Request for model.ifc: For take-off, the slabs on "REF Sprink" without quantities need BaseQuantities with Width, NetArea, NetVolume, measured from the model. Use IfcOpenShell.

First a look at what the model holds.

```python
import ifcopenshell
import ifcopenshell.util.element
import ifcopenshell.util.unit

model = ifcopenshell.open("model.ifc")
print(model.schema)
for unit_type in ("LENGTHUNIT", "AREAUNIT", "VOLUMEUNIT"):
    print(unit_type, ifcopenshell.util.unit.calculate_unit_scale(model, unit_type))
storey = next(s for s in model.by_type("IfcBuildingStorey") if s.Name == "REF Sprink")
slabs = [e for e in ifcopenshell.util.element.get_decomposition(storey) if e.is_a("IfcSlab")]
for e in sorted(slabs, key=lambda e: e.id()):
    print(e.id(), e.is_a(), e.Name, list(ifcopenshell.util.element.get_psets(e, qtos_only=True)), sep=" | ")
```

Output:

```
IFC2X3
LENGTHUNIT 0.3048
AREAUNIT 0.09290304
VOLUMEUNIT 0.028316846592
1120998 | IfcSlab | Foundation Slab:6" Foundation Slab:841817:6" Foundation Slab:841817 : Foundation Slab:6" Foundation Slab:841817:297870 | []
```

```python
import ifcopenshell
import ifcopenshell.api.pset
import ifcopenshell.geom
import ifcopenshell.util.element
import ifcopenshell.util.shape
import ifcopenshell.util.unit

model = ifcopenshell.open("model.ifc")
unit_scale = ifcopenshell.util.unit.calculate_unit_scale(model)
area_scale = ifcopenshell.util.unit.calculate_unit_scale(model, "AREAUNIT")
volume_scale = ifcopenshell.util.unit.calculate_unit_scale(model, "VOLUMEUNIT")
settings = ifcopenshell.geom.settings()

storey = next(s for s in model.by_type("IfcBuildingStorey") if s.Name == "REF Sprink")
slabs = [e for e in ifcopenshell.util.element.get_decomposition(storey) if e.is_a("IfcSlab")]

for e in sorted(slabs, key=lambda e: e.id()):
    if ifcopenshell.util.element.get_psets(e, qtos_only=True, should_inherit=False):
        continue
    # Geometry comes back in metres, in the element's own axes.
    shape = ifcopenshell.geom.create_shape(settings, e)
    values = {
        "Width": ifcopenshell.util.shape.get_z(shape.geometry) / unit_scale,
        "NetArea": ifcopenshell.util.shape.get_footprint_area(shape.geometry) / area_scale,
        "NetVolume": ifcopenshell.util.shape.get_volume(shape.geometry) / volume_scale,
    }
    qto = ifcopenshell.api.pset.add_qto(model, product=e, name="BaseQuantities")
    ifcopenshell.api.pset.edit_qto(model, qto=qto, properties=values)
    print(e.id(), {k: round(v, 3) for k, v in values.items()})

model.write("model_updated.ifc")
```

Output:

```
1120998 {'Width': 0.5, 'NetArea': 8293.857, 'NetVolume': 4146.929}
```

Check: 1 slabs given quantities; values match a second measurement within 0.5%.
